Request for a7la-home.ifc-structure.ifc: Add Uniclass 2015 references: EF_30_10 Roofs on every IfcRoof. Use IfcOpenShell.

First a look at what the model holds.

```python
import ifcopenshell

model = ifcopenshell.open("a7la-home.ifc-structure.ifc")
print(model.schema)
print("classifications:", [c.Name for c in model.by_type("IfcClassification")])
for ifc_class in ("IfcDoor", "IfcRoof", "IfcStair", "IfcWall", "IfcWindow"):
    print(ifc_class, len(model.by_type(ifc_class)))
```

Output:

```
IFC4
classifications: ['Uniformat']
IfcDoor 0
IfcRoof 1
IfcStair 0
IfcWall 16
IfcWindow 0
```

```python
import ifcopenshell
import ifcopenshell.api.classification

model = ifcopenshell.open("a7la-home.ifc-structure.ifc")

system = ifcopenshell.api.classification.add_classification(model, classification="Uniclass 2015")

codes = {
    "IfcRoof": ("EF_30_10", "Roofs"),
}
for ifc_class, (code, name) in codes.items():
    products = model.by_type(ifc_class)
    ifcopenshell.api.classification.add_reference(
        model, products=products, classification=system, identification=code, name=name
    )
    print(code, len(products))

model.write("a7la-home.ifc-structure_v2.ifc")
```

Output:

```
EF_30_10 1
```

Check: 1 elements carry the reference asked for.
